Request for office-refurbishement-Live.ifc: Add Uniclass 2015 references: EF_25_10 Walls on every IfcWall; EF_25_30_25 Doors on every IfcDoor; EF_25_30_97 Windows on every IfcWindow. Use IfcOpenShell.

First a look at what the model holds.

```python
import ifcopenshell

model = ifcopenshell.open("office-refurbishement-Live.ifc")
print(model.schema)
print("classifications:", [c.Name for c in model.by_type("IfcClassification")])
for ifc_class in ("IfcDoor", "IfcRoof", "IfcStair", "IfcWall", "IfcWindow"):
    print(ifc_class, len(model.by_type(ifc_class)))
```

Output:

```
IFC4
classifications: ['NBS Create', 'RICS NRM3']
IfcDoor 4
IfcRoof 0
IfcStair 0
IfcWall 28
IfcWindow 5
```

```python
import ifcopenshell
import ifcopenshell.api.classification

model = ifcopenshell.open("office-refurbishement-Live.ifc")

system = ifcopenshell.api.classification.add_classification(model, classification="Uniclass 2015")

codes = {
    "IfcWall": ("EF_25_10", "Walls"),
    "IfcDoor": ("EF_25_30_25", "Doors"),
    "IfcWindow": ("EF_25_30_97", "Windows"),
}
for ifc_class, (code, name) in codes.items():
    products = model.by_type(ifc_class)
    ifcopenshell.api.classification.add_reference(
        model, products=products, classification=system, identification=code, name=name
    )
    print(code, len(products))

model.write("office-refurbishement-Live_updated.ifc")
```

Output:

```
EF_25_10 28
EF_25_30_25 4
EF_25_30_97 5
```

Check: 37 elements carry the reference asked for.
